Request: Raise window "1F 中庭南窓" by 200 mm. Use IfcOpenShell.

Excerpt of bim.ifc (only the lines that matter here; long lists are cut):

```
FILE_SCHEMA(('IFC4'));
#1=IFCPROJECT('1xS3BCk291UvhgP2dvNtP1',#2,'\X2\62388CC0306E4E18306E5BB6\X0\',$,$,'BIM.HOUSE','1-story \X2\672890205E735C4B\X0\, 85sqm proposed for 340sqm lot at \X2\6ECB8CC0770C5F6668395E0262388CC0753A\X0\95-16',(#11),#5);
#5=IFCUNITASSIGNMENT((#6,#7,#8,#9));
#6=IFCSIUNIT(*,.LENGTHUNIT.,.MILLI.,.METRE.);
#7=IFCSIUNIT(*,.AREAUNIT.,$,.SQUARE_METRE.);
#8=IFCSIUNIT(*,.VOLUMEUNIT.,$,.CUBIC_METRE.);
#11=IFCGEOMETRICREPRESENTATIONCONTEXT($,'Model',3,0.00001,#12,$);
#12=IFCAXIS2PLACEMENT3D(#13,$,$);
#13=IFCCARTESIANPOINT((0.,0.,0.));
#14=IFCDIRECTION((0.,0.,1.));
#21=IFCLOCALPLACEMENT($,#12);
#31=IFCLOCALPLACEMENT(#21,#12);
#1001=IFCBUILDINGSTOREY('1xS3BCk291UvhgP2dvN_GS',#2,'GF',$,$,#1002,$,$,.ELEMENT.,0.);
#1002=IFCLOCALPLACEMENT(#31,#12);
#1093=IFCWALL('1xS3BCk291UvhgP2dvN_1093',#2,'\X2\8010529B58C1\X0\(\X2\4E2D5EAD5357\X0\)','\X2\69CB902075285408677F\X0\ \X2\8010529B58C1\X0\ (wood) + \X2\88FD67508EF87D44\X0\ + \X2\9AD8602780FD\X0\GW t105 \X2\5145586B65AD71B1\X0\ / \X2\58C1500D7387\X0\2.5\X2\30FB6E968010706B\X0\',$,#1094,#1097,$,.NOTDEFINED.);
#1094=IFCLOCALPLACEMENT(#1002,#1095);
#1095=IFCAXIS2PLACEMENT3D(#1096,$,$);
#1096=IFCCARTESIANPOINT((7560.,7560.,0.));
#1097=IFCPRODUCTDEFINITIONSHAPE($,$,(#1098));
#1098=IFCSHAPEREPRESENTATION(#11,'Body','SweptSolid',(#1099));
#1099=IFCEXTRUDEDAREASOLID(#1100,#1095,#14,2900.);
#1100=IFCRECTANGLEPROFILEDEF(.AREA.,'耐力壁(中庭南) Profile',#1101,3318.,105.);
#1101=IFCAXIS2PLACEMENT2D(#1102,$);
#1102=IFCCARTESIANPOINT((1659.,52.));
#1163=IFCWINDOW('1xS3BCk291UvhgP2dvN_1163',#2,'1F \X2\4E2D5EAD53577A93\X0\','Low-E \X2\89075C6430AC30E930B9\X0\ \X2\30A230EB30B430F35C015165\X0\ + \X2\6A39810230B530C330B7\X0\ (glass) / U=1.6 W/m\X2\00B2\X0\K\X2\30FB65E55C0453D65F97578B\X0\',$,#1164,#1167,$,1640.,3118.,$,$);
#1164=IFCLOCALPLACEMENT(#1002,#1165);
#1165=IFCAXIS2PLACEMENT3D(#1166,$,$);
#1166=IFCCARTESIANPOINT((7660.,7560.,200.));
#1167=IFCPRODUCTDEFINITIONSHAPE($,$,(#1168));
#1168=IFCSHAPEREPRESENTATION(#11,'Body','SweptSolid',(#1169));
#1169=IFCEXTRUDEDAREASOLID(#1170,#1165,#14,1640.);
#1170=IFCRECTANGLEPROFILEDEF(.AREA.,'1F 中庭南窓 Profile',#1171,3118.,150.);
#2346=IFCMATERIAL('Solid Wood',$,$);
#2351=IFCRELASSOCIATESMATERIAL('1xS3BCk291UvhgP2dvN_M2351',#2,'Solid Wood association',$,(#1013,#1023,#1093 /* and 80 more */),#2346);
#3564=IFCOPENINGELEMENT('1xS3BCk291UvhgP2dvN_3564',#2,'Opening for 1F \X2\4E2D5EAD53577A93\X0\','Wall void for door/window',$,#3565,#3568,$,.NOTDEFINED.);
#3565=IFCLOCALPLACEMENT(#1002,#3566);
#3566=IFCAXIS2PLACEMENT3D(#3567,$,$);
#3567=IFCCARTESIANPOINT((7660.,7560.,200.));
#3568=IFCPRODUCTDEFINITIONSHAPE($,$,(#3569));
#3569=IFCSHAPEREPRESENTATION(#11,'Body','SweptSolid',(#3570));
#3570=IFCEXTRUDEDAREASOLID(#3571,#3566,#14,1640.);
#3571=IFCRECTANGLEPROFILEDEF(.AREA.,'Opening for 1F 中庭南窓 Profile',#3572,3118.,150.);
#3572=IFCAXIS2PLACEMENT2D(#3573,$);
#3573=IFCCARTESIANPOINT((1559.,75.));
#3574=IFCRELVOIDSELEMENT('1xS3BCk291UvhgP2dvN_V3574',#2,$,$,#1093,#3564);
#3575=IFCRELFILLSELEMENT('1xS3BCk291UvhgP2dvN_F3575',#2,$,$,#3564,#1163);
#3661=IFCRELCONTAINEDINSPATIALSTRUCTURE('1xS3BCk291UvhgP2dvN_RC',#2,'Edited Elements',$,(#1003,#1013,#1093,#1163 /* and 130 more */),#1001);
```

```python
import numpy as np
import ifcopenshell
import ifcopenshell.api.geometry
import ifcopenshell.util.placement
import ifcopenshell.util.unit

model = ifcopenshell.open("bim.ifc")
unit_scale = ifcopenshell.util.unit.calculate_unit_scale(model)

window = model.by_guid("1xS3BCk291UvhgP2dvN_1163")
opening = window.FillsVoids[0].RelatingOpeningElement
dz = 200.0

shift = np.array([0.0, 0.0, dz])
# The window is not placed relative to its opening, so move both.
for product in (opening, window):
    matrix = ifcopenshell.util.placement.get_local_placement(product.ObjectPlacement)
    matrix[:3, 3] += shift
    ifcopenshell.api.geometry.edit_object_placement(model, product=product, matrix=matrix, is_si=False)

print(f"moved by {dz * unit_scale:+.3f} m")

model.write("bim_updated.ifc")
```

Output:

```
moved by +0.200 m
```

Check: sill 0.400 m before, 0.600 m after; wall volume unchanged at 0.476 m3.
